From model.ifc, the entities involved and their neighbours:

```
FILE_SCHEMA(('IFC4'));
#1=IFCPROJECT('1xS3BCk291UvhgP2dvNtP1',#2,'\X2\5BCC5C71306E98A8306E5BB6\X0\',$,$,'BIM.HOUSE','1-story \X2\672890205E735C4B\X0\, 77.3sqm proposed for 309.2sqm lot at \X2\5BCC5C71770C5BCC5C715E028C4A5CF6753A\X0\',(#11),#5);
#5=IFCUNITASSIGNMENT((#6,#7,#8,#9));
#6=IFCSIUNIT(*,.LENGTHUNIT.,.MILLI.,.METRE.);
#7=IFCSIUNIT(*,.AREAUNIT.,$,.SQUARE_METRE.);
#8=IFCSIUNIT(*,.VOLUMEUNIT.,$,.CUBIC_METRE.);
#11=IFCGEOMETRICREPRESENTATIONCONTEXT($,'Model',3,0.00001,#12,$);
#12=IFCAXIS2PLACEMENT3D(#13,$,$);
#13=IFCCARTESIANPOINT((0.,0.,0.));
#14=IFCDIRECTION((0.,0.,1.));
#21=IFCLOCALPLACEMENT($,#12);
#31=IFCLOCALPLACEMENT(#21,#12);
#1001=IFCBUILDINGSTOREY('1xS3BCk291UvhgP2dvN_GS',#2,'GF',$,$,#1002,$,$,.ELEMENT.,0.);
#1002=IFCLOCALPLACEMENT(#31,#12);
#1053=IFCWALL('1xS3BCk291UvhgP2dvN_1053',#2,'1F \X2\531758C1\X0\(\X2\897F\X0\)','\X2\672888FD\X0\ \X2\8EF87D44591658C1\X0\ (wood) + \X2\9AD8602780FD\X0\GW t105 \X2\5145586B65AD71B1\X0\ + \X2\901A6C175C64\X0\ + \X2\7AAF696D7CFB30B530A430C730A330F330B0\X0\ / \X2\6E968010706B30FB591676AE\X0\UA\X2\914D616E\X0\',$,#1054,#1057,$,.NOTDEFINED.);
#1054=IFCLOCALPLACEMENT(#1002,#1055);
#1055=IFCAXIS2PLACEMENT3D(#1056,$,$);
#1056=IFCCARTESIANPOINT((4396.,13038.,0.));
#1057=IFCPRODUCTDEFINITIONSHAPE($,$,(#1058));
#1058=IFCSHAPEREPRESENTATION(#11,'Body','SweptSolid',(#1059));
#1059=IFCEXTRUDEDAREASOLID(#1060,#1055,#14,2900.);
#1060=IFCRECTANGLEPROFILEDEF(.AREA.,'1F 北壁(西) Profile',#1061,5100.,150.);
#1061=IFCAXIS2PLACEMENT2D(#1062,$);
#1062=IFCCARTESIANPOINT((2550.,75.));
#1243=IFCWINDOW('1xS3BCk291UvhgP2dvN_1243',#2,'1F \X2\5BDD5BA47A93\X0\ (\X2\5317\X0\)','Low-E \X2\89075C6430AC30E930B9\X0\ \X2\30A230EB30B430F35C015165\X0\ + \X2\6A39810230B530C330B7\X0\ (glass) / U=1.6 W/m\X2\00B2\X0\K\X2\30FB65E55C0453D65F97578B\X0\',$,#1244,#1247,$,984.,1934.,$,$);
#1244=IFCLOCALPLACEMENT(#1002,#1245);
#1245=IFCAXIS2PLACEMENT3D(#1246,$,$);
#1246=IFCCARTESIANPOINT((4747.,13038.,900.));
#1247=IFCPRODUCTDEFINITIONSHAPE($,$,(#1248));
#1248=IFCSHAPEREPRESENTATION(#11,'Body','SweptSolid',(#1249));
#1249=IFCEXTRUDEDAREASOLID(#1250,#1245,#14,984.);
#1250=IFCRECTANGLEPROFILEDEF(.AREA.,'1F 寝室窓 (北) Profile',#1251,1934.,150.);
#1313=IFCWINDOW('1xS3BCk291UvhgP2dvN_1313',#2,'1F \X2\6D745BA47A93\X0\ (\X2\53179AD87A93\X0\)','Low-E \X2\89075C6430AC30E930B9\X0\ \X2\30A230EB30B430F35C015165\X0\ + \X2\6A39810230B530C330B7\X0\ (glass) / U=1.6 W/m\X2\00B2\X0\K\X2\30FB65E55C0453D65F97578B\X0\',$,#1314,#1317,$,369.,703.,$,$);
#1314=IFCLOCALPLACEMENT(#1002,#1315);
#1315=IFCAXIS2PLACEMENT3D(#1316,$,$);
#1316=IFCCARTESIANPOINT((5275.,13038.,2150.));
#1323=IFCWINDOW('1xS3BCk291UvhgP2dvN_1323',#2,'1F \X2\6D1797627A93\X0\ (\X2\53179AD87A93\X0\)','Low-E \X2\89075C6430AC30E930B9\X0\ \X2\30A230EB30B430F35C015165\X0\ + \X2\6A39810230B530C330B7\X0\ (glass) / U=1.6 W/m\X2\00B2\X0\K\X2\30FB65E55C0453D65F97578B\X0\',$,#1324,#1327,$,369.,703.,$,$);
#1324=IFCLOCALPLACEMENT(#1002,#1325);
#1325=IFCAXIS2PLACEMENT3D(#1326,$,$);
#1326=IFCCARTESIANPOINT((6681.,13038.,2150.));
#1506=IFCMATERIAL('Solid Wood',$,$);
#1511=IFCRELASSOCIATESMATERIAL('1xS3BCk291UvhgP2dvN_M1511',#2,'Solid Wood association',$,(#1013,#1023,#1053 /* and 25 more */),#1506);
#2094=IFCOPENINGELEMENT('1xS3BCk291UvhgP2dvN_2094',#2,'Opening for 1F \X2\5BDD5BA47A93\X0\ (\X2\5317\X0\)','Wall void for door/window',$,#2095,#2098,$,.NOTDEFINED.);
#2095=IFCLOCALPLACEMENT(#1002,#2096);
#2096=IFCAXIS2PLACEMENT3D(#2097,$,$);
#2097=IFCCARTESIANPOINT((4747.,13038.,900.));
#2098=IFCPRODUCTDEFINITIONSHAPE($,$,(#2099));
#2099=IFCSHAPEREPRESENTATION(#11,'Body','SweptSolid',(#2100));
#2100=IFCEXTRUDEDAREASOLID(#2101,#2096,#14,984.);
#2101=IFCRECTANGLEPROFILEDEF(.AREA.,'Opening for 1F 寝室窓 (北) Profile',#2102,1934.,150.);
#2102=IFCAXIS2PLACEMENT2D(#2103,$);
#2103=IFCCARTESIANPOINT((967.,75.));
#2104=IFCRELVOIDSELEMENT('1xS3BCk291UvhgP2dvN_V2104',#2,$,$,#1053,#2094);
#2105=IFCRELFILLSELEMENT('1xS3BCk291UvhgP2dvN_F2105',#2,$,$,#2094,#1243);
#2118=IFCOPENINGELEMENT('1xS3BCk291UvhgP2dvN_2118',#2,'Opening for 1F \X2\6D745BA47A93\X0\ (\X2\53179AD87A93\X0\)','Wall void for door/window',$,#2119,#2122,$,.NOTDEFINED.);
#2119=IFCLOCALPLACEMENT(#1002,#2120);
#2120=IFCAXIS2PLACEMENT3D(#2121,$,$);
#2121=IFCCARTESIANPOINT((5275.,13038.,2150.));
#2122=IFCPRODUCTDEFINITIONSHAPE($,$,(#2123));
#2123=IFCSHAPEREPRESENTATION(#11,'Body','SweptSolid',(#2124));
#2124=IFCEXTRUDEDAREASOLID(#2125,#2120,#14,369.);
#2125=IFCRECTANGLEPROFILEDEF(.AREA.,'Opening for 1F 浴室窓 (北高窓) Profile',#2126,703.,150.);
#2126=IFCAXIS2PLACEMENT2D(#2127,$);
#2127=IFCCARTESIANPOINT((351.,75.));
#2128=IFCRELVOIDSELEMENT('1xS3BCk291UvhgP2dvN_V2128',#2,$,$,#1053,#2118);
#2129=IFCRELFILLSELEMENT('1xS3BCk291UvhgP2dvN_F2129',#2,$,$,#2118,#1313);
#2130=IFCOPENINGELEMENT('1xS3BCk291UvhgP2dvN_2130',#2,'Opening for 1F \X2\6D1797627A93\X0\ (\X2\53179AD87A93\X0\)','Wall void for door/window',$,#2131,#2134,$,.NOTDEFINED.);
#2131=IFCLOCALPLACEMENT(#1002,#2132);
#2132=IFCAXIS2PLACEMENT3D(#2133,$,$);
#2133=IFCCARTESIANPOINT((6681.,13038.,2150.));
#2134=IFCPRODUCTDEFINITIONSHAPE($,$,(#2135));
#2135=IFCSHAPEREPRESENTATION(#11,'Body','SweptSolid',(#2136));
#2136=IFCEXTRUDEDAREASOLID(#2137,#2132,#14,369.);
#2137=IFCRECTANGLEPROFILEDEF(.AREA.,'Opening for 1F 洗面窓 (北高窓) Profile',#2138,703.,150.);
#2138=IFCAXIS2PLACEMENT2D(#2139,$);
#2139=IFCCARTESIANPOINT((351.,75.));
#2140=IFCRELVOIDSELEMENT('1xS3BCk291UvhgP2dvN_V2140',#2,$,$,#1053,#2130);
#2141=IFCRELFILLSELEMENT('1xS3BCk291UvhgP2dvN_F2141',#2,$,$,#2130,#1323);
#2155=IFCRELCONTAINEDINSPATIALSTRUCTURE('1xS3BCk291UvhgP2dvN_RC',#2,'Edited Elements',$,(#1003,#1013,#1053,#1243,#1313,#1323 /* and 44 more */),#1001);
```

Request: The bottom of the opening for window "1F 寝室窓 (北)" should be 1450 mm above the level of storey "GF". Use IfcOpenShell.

```python
import numpy as np
import ifcopenshell
import ifcopenshell.api.geometry
import ifcopenshell.geom
import ifcopenshell.util.element
import ifcopenshell.util.placement
import ifcopenshell.util.shape
import ifcopenshell.util.unit

model = ifcopenshell.open("model.ifc")
unit_scale = ifcopenshell.util.unit.calculate_unit_scale(model)

window = model.by_guid("1xS3BCk291UvhgP2dvN_1243")
opening = window.FillsVoids[0].RelatingOpeningElement
storey = ifcopenshell.util.element.get_container(window, ifc_class="IfcBuildingStorey")
level = ifcopenshell.util.placement.get_local_placement(storey.ObjectPlacement)[2, 3]

# The opening's origin need not be at the sill, so measure its lowest point.
shape = ifcopenshell.geom.create_shape(ifcopenshell.geom.settings(), opening)
bottom = ifcopenshell.util.shape.get_shape_bottom_elevation(shape, shape.geometry) / unit_scale
dz = level + 1450.0 - bottom

shift = np.array([0.0, 0.0, dz])
# The window is not placed relative to its opening, so move both.
for product in (opening, window):
    matrix = ifcopenshell.util.placement.get_local_placement(product.ObjectPlacement)
    matrix[:3, 3] += shift
    ifcopenshell.api.geometry.edit_object_placement(model, product=product, matrix=matrix, is_si=False)

print(f"moved by {dz * unit_scale:+.3f} m")

model.write("model_rev.ifc")
```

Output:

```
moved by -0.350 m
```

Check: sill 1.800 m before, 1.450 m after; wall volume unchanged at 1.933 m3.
